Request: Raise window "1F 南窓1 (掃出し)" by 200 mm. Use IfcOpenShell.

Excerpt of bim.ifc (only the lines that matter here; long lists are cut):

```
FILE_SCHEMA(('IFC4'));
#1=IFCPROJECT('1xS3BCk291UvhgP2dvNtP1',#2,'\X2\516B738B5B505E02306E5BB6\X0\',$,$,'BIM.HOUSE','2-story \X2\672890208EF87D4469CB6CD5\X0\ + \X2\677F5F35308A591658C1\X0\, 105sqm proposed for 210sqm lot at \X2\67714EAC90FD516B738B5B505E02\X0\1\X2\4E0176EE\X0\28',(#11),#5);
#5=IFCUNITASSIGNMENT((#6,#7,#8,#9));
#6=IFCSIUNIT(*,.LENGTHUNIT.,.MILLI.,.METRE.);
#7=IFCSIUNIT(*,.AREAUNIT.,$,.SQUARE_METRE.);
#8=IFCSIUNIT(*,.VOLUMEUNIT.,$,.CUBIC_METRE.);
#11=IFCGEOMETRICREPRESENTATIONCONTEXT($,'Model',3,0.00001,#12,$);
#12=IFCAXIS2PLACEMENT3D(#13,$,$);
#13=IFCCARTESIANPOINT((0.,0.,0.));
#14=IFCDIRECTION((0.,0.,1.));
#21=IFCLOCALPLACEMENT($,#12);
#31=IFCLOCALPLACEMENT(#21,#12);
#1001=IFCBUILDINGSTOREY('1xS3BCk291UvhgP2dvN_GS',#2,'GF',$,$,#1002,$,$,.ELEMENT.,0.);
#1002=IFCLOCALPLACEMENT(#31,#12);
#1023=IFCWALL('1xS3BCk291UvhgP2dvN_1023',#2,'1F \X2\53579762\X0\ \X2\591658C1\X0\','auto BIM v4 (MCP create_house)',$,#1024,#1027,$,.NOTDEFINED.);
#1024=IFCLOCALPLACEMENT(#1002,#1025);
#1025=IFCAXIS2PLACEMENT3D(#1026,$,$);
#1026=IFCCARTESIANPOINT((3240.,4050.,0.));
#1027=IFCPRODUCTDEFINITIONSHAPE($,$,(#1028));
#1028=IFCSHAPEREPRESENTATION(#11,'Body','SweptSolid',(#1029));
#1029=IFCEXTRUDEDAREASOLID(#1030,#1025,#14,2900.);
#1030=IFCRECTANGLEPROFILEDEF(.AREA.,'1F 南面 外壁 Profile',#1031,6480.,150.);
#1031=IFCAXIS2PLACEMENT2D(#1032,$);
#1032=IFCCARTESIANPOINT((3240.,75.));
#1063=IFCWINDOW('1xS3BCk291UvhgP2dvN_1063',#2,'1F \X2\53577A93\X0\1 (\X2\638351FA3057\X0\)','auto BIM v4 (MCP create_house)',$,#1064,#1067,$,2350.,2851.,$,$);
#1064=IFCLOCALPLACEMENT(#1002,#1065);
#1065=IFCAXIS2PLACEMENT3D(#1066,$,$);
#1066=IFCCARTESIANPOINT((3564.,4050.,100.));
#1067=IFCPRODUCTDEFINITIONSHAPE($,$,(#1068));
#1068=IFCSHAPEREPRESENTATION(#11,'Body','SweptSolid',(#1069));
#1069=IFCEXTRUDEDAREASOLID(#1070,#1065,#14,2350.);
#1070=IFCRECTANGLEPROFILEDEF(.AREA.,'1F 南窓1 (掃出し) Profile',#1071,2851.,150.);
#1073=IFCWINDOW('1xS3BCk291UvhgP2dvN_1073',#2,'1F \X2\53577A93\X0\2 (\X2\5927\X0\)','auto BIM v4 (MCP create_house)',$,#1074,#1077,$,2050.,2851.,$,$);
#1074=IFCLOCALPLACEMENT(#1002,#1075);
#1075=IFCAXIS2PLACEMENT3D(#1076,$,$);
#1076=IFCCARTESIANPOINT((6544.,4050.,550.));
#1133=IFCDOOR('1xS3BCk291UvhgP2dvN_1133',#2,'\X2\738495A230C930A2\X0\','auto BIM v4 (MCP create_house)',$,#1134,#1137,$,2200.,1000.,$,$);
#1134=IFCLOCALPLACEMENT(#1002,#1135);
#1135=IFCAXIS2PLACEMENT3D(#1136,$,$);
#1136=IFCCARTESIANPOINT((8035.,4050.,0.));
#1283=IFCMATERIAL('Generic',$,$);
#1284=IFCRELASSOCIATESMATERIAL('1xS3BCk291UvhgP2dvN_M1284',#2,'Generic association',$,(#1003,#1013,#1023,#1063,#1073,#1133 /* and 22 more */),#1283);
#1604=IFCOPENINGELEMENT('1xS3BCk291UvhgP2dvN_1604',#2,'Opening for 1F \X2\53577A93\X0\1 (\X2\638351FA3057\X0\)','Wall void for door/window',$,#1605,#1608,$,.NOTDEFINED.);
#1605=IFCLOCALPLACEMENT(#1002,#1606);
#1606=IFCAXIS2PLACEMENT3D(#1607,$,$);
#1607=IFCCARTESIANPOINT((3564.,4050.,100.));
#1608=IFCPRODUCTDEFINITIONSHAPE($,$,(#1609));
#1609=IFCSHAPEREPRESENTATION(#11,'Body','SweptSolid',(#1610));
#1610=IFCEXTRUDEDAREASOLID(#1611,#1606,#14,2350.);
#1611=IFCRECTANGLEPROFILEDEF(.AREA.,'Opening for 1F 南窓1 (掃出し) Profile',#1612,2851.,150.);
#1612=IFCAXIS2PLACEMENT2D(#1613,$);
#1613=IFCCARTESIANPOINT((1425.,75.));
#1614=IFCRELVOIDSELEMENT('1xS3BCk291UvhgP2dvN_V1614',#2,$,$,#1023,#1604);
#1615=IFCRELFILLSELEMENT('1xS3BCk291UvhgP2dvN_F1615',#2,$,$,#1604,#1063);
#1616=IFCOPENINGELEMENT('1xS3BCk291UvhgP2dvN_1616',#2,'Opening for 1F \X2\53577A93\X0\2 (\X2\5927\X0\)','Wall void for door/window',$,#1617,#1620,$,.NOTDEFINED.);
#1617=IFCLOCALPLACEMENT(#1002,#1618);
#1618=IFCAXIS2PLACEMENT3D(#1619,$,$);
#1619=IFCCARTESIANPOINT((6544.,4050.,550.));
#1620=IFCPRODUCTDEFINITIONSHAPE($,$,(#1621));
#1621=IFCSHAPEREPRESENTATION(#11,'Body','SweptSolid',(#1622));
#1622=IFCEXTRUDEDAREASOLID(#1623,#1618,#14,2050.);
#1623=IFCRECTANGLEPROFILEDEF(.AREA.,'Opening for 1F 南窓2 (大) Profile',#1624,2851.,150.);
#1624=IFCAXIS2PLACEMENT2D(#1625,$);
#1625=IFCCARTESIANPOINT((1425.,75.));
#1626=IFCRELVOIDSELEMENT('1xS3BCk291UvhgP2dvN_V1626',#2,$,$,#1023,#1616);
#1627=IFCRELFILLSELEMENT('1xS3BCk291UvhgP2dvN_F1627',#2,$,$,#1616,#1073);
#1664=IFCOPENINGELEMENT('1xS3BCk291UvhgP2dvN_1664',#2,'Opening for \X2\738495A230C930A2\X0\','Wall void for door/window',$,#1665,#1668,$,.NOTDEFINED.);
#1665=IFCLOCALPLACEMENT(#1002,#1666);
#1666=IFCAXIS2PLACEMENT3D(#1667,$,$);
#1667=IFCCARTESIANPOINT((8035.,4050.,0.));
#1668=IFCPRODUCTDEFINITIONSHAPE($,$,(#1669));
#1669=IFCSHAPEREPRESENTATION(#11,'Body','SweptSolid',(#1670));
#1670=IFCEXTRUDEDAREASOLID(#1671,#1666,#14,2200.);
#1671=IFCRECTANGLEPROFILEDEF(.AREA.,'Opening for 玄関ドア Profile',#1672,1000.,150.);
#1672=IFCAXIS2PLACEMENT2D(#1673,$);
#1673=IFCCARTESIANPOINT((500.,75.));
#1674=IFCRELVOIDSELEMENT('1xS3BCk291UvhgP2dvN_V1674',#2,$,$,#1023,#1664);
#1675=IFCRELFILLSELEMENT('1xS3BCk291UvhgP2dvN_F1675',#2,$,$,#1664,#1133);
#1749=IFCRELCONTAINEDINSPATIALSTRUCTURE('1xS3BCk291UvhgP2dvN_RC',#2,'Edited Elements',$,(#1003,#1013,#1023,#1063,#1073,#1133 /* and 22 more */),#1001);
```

```python
import numpy as np
import ifcopenshell
import ifcopenshell.api.geometry
import ifcopenshell.util.placement
import ifcopenshell.util.unit

model = ifcopenshell.open("bim.ifc")
unit_scale = ifcopenshell.util.unit.calculate_unit_scale(model)

window = model.by_guid("1xS3BCk291UvhgP2dvN_1063")
opening = window.FillsVoids[0].RelatingOpeningElement
dz = 200.0

shift = np.array([0.0, 0.0, dz])
# The window is not placed relative to its opening, so move both.
for product in (opening, window):
    matrix = ifcopenshell.util.placement.get_local_placement(product.ObjectPlacement)
    matrix[:3, 3] += shift
    ifcopenshell.api.geometry.edit_object_placement(model, product=product, matrix=matrix, is_si=False)

print(f"moved by {dz * unit_scale:+.3f} m")

model.write("bim-out.ifc")
```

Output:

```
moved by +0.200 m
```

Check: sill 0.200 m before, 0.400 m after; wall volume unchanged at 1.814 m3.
